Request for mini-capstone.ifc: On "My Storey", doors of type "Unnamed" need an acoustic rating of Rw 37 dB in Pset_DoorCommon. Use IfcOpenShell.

First a look at what the model holds.

```python
import ifcopenshell
import ifcopenshell.util.element

model = ifcopenshell.open("mini-capstone.ifc")
print(model.schema)
storey = next(s for s in model.by_type("IfcBuildingStorey") if s.Name == "My Storey")
doors = [e for e in ifcopenshell.util.element.get_decomposition(storey) if e.is_a("IfcDoor")]
seen = {}
for e in doors:
    element_type = ifcopenshell.util.element.get_type(e)
    key = (element_type.Name if element_type != e and element_type else None, ifcopenshell.util.element.get_pset(e, "Pset_DoorCommon", "AcousticRating"))
    seen[key] = seen.get(key, 0) + 1
for (name, value), count in sorted(seen.items(), key=str):
    print(count, "x", name, "|", value)
```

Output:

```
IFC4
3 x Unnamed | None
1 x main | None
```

```python
import ifcopenshell
import ifcopenshell.api.pset
import ifcopenshell.util.element

model = ifcopenshell.open("mini-capstone.ifc")

storey = next(s for s in model.by_type("IfcBuildingStorey") if s.Name == "My Storey")
doors = [e for e in ifcopenshell.util.element.get_decomposition(storey) if e.is_a("IfcDoor")]

count = 0
for e in doors:
    element_type = ifcopenshell.util.element.get_type(e)
    if element_type in (None, e) or element_type.Name != "Unnamed":
        continue
    # add_pset returns the element's existing set when there is one.
    pset = ifcopenshell.api.pset.add_pset(model, product=e, name="Pset_DoorCommon")
    ifcopenshell.api.pset.edit_pset(model, pset=pset, properties={"AcousticRating": "Rw 37 dB"})
    count += 1

print(count, "doors updated")

model.write("mini-capstone_rev.ifc")
```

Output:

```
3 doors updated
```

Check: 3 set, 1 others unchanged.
